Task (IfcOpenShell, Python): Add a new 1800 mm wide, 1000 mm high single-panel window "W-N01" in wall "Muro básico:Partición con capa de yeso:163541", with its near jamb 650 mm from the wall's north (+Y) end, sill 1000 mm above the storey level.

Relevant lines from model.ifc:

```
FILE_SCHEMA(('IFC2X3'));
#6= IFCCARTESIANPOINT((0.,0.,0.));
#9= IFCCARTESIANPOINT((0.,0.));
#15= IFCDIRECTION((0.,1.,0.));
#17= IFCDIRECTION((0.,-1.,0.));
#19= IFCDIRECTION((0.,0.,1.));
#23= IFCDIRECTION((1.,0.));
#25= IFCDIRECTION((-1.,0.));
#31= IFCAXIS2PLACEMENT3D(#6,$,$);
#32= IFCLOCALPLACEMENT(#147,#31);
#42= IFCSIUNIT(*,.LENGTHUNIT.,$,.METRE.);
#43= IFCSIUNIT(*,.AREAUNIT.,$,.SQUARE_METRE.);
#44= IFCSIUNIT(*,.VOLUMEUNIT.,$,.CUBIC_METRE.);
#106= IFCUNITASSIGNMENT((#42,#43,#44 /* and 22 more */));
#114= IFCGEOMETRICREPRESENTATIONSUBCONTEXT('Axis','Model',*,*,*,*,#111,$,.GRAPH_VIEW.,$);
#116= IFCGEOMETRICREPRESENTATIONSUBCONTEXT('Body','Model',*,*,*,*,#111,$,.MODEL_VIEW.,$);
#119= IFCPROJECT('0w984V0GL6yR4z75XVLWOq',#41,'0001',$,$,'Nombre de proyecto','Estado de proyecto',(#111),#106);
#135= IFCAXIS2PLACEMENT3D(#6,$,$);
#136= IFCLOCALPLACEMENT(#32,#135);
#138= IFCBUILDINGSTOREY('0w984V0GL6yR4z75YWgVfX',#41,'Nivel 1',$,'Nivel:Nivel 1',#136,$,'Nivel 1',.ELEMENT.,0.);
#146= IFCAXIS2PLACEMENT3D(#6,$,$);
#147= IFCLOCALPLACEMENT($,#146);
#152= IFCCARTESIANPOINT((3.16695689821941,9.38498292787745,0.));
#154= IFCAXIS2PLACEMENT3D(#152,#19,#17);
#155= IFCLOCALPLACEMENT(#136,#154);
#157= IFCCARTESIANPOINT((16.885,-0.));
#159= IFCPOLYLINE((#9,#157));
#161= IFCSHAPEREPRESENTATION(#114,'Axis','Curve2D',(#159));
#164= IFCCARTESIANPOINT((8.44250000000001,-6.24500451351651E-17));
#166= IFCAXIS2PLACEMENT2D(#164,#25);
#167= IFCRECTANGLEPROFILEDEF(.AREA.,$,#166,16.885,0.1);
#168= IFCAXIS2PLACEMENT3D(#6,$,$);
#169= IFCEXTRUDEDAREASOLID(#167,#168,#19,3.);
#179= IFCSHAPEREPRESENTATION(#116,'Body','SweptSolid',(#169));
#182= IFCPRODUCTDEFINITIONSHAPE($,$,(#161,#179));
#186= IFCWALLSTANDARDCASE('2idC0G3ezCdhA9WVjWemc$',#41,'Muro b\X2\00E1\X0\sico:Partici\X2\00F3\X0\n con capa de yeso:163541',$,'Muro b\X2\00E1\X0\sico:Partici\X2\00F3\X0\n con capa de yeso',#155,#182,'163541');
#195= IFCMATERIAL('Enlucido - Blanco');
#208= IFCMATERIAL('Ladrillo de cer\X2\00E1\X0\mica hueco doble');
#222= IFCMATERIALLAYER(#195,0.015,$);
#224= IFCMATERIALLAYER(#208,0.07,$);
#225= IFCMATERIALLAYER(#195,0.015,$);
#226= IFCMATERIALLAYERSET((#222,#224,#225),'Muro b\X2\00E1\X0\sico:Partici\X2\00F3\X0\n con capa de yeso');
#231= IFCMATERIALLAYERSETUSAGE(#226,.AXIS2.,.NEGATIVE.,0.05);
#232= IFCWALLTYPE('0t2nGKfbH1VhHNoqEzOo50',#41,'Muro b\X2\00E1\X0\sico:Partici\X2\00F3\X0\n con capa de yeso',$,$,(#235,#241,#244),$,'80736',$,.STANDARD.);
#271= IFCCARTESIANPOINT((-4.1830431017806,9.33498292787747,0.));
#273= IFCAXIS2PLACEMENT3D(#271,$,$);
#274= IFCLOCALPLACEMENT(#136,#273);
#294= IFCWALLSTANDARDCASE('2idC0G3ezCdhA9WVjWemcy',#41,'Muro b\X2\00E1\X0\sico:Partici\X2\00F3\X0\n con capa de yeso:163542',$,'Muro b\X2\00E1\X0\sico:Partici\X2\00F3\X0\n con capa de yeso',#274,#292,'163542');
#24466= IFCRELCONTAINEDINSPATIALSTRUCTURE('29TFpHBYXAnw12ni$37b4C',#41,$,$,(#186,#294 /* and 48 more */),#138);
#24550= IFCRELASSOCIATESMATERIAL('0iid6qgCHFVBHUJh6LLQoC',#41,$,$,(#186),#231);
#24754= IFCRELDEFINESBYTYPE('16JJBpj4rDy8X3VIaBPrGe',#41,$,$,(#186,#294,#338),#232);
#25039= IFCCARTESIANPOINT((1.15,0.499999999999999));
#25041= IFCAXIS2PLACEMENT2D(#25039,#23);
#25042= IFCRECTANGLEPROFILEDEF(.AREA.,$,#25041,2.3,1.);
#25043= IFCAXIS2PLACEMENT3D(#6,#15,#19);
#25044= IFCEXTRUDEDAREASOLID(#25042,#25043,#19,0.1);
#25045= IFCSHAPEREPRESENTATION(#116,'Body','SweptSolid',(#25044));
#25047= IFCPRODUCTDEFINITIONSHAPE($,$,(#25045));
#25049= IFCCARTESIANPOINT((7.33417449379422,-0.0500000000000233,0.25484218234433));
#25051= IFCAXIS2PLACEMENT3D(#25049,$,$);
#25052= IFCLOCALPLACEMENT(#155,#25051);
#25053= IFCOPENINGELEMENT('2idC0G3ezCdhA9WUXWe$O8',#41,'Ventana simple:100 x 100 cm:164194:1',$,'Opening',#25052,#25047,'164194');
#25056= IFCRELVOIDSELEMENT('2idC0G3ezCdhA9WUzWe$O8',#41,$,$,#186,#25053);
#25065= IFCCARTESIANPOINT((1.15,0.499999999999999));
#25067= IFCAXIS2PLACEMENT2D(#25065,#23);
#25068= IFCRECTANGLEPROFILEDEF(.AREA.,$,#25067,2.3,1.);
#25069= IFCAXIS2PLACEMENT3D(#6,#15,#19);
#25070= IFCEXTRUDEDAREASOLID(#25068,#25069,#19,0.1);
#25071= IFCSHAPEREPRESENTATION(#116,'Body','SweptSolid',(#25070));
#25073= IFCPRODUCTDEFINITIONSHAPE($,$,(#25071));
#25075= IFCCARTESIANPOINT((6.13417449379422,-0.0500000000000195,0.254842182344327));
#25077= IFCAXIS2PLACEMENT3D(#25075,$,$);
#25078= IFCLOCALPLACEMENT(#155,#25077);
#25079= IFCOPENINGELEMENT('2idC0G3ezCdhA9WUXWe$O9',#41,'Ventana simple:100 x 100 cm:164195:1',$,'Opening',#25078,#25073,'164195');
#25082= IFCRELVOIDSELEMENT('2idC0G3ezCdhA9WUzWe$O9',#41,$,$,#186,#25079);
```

```python
import numpy as np
import ifcopenshell
import ifcopenshell.api.feature
import ifcopenshell.api.geometry
import ifcopenshell.api.root
import ifcopenshell.api.spatial
import ifcopenshell.api.type
import ifcopenshell.geom
import ifcopenshell.util.element
import ifcopenshell.util.placement
import ifcopenshell.util.representation
import ifcopenshell.util.shape
import ifcopenshell.util.unit

model = ifcopenshell.open("model.ifc")
unit_scale = ifcopenshell.util.unit.calculate_unit_scale(model)
settings = ifcopenshell.geom.settings()


def volume(element):
    """Net volume in cubic metres, openings subtracted."""
    shape = ifcopenshell.geom.create_shape(settings, element)
    return ifcopenshell.util.shape.get_volume(shape.geometry)


wall = model.by_id(186)
storey = ifcopenshell.util.element.get_container(wall, ifc_class="IfcBuildingStorey")
context = ifcopenshell.util.representation.get_context(model, "Model", "Body", "MODEL_VIEW")
before = volume(wall)

width, height, from_end, sill = 1.8, 1, 0.65, 1  # metres

# The wall runs along its own X axis, and the end named is its -X end.
wall_shape = ifcopenshell.geom.create_shape(settings, wall)
x, y, z = ifcopenshell.util.shape.get_vertices(wall_shape.geometry).T
start = x.min() + from_end
face, thickness = float(y.min()), float(y.max() - y.min())
wall_matrix = ifcopenshell.util.placement.get_local_placement(wall.ObjectPlacement)
level = ifcopenshell.util.placement.get_local_placement(storey.ObjectPlacement)[2, 3]


def in_wall(x, y):
    """Placement at x, y metres in the wall's axes, at sill height."""
    matrix = wall_matrix.copy()
    matrix[:, 3] = wall_matrix @ np.array([x / unit_scale, y / unit_scale, 0.0, 1.0])
    matrix[2, 3] = level + sill / unit_scale
    return matrix


# Opening: a box that overshoots both wall faces by 50 mm.
opening = ifcopenshell.api.root.create_entity(model, ifc_class="IfcOpeningElement")
box = ifcopenshell.api.geometry.add_wall_representation(
    model, context=context, length=width, height=height, thickness=thickness + 0.1
)
ifcopenshell.api.geometry.assign_representation(model, product=opening, representation=box)
ifcopenshell.api.geometry.edit_object_placement(model, product=opening, matrix=in_wall(start, face - 0.05), is_si=False)
ifcopenshell.api.feature.add_feature(model, feature=opening, element=wall)

window = ifcopenshell.api.root.create_entity(model, ifc_class="IfcWindow", name="W-N01")
window.OverallWidth, window.OverallHeight = width / unit_scale, height / unit_scale
body = ifcopenshell.api.geometry.add_window_representation(
    model,
    context=context,
    overall_width=window.OverallWidth,
    overall_height=window.OverallHeight,
    partition_type="SINGLE_PANEL",
)
ifcopenshell.api.geometry.assign_representation(model, product=window, representation=body)
ifcopenshell.api.spatial.assign_container(model, products=[window], relating_structure=storey)
fills = ifcopenshell.api.feature.add_filling(model, opening=opening, element=window)
fills.OwnerHistory = window.OwnerHistory  # required in IFC2X3

# IFC2X3 keeps the operation on the window style.
style = ifcopenshell.api.root.create_entity(model, ifc_class="IfcWindowStyle", name="W-N01")
style.OperationType, style.ConstructionType = "SINGLE_PANEL", "NOTDEFINED"
style.ParameterTakesPrecedence = style.Sizeable = False
ifcopenshell.api.type.assign_type(model, related_objects=[window], relating_type=style)

# Centre the window in the wall's thickness.
ifcopenshell.api.geometry.edit_object_placement(model, product=window, matrix=in_wall(start, face), is_si=False)
window_shape = ifcopenshell.geom.create_shape(settings, window)
depth = ifcopenshell.util.shape.get_vertices(window_shape.geometry)[:, 1]
offset = face + thickness / 2 - (depth.min() + depth.max()) / 2
ifcopenshell.api.geometry.edit_object_placement(model, product=window, matrix=in_wall(start, offset), is_si=False)

after = volume(wall)

print(f"wall volume {before:.3f} -> {after:.3f} m3")

model.write("model_updated.ifc")
```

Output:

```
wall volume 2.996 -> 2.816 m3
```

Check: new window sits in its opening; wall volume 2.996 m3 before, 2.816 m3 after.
